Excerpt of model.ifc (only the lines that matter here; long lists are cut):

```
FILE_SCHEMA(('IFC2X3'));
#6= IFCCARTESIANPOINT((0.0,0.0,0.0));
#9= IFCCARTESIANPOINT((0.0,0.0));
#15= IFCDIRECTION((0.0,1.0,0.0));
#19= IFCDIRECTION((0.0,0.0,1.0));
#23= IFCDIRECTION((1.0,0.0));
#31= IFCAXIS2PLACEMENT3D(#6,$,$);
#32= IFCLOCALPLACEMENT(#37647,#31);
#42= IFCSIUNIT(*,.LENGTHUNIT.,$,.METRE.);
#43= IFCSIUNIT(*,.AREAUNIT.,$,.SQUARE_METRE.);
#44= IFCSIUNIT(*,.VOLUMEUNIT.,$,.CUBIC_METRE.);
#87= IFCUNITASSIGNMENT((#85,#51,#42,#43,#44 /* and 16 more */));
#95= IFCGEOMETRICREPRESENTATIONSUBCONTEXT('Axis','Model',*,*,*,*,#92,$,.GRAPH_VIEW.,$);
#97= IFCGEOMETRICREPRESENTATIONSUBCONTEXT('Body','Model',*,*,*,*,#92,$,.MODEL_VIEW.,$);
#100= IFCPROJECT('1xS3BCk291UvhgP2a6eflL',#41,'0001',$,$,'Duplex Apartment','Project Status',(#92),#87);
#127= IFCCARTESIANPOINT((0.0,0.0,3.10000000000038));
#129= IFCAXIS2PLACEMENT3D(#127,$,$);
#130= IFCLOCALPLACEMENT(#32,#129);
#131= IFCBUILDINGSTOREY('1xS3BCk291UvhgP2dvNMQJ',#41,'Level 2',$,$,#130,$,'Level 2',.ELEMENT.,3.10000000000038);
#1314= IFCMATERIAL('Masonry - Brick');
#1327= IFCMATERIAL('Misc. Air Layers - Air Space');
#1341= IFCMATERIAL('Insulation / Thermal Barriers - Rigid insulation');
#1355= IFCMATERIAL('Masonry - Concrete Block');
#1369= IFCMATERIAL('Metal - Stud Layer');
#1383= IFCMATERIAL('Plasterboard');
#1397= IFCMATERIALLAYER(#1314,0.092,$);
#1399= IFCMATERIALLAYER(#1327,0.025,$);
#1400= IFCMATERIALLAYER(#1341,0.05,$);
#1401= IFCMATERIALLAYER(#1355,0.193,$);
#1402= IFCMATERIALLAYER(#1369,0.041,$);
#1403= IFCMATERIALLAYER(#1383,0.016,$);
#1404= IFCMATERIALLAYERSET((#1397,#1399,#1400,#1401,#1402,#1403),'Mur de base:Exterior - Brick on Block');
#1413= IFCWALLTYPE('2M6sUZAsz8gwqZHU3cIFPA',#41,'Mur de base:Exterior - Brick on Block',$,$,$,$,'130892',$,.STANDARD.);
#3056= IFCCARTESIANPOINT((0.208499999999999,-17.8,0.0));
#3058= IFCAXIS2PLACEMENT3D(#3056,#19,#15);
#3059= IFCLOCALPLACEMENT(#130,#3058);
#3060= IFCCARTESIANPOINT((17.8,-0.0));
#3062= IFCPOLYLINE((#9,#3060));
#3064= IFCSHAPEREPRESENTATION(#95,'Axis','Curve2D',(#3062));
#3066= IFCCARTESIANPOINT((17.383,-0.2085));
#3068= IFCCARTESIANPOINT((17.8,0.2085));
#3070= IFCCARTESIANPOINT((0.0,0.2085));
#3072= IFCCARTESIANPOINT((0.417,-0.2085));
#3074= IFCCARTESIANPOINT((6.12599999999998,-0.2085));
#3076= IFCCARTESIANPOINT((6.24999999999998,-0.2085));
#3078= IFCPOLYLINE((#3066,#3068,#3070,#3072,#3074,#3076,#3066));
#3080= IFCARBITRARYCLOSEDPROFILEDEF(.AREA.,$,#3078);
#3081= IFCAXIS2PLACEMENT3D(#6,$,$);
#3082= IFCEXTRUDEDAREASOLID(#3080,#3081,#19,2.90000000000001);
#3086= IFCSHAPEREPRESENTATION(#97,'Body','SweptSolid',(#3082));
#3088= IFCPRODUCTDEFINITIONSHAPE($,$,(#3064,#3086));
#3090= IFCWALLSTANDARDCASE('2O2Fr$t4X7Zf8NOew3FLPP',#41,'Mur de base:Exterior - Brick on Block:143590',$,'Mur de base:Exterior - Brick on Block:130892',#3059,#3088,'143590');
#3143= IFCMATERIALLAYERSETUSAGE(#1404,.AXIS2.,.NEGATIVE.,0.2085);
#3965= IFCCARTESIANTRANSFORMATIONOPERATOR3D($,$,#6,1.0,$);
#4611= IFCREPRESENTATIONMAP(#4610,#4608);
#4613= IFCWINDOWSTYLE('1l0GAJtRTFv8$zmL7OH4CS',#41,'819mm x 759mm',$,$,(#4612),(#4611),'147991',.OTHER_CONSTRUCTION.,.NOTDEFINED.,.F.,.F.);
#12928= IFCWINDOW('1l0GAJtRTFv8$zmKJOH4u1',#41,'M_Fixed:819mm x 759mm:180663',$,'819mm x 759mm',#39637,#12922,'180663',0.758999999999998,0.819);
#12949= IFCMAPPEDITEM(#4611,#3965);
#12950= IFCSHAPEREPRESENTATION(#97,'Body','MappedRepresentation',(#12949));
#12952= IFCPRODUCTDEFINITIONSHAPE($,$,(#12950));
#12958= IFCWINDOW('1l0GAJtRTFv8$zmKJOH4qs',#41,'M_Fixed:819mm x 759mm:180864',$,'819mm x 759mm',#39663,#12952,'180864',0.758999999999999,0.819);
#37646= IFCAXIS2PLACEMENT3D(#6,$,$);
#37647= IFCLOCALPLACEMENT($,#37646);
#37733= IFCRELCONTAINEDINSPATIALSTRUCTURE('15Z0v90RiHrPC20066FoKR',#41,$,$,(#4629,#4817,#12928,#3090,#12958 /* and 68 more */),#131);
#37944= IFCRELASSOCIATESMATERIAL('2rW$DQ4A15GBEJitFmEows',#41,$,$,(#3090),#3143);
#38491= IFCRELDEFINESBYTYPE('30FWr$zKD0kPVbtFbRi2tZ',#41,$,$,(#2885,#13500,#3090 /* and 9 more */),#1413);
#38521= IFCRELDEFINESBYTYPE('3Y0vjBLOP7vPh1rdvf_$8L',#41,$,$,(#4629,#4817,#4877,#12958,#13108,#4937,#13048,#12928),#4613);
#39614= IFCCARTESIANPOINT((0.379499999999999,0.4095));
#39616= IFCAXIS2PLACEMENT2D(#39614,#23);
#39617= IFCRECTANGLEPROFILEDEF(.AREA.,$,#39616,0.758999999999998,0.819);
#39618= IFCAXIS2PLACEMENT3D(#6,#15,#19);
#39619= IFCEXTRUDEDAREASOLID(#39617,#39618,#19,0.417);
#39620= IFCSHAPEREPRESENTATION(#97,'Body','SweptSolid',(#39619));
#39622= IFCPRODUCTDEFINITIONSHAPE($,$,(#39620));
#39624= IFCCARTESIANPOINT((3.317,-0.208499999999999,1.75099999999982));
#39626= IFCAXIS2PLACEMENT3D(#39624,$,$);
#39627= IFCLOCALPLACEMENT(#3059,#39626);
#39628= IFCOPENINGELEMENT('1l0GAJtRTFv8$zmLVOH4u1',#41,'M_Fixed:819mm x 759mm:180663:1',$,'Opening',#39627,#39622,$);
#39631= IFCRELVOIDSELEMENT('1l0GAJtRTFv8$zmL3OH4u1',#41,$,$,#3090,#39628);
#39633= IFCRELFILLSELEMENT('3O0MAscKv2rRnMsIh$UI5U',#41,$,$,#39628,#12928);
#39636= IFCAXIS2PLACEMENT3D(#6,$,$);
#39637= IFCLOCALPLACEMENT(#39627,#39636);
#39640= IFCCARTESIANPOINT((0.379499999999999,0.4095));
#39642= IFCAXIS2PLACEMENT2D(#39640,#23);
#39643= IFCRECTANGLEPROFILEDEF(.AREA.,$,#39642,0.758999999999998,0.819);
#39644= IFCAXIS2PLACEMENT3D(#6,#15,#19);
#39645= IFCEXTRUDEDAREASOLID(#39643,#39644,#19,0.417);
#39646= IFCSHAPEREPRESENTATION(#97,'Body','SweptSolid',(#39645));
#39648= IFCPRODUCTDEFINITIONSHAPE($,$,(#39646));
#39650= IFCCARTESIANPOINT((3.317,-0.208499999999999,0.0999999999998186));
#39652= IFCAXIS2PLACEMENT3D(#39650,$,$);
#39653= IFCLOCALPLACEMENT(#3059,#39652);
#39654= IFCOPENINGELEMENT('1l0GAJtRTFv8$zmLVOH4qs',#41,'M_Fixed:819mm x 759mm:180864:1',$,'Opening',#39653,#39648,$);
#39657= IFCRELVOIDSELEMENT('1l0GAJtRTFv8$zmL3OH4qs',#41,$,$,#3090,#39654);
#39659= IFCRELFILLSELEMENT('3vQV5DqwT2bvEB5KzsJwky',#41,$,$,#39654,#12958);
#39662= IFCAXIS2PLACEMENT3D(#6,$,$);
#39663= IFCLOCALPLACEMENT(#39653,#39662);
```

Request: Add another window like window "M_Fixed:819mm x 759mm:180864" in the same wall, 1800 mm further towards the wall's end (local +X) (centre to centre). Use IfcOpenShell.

```python
import ifcopenshell
import ifcopenshell.api.feature
import ifcopenshell.api.geometry
import ifcopenshell.api.root
import ifcopenshell.geom
import ifcopenshell.util.element
import ifcopenshell.util.placement
import ifcopenshell.util.shape

model = ifcopenshell.open("model.ifc")
settings = ifcopenshell.geom.settings()


def volume(element):
    """Net volume in cubic metres, openings subtracted."""
    shape = ifcopenshell.geom.create_shape(settings, element)
    return ifcopenshell.util.shape.get_volume(shape.geometry)


def reuse_history(source, copy):
    """copy_class also copies each property set's owner history, people and application; keep the originals."""
    for rel in copy.IsDefinedBy:
        if rel.is_a("IfcRelDefinesByProperties") and (history := rel.RelatingPropertyDefinition.OwnerHistory):
            rel.RelatingPropertyDefinition.OwnerHistory = source.OwnerHistory
            ifcopenshell.util.element.remove_deep2(model, history)


window = model.by_id(12958)
opening = window.FillsVoids[0].RelatingOpeningElement
wall = opening.VoidsElements[0].RelatingBuildingElement
before = volume(wall)
shift = ifcopenshell.util.placement.get_local_placement(wall.ObjectPlacement)[:3, 0] * 1.8

# copy_class copies the void relationship, type, container and properties, but no geometry.
new_opening = ifcopenshell.api.root.copy_class(model, product=opening)
new_opening.Representation = ifcopenshell.util.element.copy_deep(
    model, opening.Representation, exclude=["IfcGeometricRepresentationContext", "IfcRepresentationMap"]
)
new_opening.Name = "M_Fixed:819mm x 759mm"
new_window = ifcopenshell.api.root.copy_class(model, product=window)
new_window.Representation = ifcopenshell.util.element.copy_deep(
    model, window.Representation, exclude=["IfcGeometricRepresentationContext", "IfcRepresentationMap"]
)
new_window.Name = "M_Fixed:819mm x 759mm"
new_window.Tag = None
reuse_history(window, new_window)
fills = ifcopenshell.api.feature.add_filling(model, opening=new_opening, element=new_window)
fills.OwnerHistory = new_window.OwnerHistory  # required in IFC2X3

for old, new in ((opening, new_opening), (window, new_window)):
    matrix = ifcopenshell.util.placement.get_local_placement(old.ObjectPlacement)
    matrix[:3, 3] += shift
    ifcopenshell.api.geometry.edit_object_placement(model, product=new, matrix=matrix, is_si=False)

after = volume(wall)

print(f"wall volume {before:.3f} -> {after:.3f} m3")

model.write("model_updated.ifc")
```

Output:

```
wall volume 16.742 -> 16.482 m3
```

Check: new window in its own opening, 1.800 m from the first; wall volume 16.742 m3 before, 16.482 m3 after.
